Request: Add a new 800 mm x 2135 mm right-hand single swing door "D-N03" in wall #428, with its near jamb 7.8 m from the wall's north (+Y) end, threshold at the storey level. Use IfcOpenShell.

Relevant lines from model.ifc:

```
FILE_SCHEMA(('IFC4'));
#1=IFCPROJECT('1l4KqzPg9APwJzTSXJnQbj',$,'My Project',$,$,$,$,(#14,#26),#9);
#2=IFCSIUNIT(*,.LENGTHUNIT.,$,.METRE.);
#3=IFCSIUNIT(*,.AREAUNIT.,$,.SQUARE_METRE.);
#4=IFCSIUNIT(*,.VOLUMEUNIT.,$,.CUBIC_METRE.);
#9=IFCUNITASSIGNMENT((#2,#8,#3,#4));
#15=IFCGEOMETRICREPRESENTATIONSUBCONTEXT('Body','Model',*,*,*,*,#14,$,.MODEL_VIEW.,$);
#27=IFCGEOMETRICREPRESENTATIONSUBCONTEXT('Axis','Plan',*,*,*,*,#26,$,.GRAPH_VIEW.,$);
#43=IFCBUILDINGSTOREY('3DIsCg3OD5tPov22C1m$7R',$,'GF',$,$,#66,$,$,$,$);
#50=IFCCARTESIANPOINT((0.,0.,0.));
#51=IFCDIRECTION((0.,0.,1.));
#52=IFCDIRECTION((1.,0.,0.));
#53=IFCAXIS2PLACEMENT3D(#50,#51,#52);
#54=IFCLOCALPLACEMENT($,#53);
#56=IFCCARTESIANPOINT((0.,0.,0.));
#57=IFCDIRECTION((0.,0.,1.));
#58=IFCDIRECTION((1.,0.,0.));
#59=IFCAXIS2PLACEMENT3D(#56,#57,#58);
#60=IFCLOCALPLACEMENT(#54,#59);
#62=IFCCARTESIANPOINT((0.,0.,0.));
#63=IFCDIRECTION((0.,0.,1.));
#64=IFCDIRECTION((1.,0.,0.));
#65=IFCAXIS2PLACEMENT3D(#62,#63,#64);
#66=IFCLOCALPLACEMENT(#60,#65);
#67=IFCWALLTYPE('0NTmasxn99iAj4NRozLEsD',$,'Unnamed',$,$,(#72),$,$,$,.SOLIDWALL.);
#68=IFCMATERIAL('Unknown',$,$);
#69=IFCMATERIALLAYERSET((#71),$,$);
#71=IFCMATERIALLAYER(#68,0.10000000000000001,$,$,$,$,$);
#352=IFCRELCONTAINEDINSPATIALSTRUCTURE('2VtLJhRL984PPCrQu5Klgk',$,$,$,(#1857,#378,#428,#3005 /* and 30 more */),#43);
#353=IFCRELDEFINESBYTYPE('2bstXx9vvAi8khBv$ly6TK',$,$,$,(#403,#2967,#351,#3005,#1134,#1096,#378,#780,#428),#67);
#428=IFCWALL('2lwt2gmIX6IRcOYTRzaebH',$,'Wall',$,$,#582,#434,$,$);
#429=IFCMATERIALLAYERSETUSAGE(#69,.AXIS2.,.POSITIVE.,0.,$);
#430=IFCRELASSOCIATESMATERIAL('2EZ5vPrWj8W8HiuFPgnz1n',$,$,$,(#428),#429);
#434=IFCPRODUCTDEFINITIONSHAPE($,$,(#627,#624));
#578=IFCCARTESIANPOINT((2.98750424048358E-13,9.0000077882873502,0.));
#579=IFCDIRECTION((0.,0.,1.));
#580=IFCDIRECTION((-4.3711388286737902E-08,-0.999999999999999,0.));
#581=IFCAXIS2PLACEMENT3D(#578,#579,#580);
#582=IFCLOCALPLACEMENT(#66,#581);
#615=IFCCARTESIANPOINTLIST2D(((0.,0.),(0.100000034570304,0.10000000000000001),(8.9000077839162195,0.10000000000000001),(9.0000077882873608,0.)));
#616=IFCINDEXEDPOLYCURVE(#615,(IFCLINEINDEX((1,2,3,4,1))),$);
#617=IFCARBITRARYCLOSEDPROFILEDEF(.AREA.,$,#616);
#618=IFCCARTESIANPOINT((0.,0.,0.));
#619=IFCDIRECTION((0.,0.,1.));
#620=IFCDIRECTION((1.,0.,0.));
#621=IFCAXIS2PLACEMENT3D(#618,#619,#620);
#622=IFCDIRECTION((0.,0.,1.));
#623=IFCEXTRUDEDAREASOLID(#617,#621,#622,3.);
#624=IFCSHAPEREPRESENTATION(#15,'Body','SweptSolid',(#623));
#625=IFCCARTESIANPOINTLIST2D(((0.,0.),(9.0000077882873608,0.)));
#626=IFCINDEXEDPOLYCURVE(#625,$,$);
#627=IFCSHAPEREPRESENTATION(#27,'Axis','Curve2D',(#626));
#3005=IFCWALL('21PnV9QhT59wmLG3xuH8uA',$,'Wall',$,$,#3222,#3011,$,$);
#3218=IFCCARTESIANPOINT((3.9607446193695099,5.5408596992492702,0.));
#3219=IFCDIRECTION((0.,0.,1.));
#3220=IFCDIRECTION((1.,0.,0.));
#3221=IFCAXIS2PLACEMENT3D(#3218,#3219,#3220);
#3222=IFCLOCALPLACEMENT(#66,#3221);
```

```python
import numpy as np
import ifcopenshell
import ifcopenshell.api.feature
import ifcopenshell.api.geometry
import ifcopenshell.api.root
import ifcopenshell.api.spatial
import ifcopenshell.geom
import ifcopenshell.util.element
import ifcopenshell.util.placement
import ifcopenshell.util.representation
import ifcopenshell.util.shape
import ifcopenshell.util.unit

model = ifcopenshell.open("model.ifc")
unit_scale = ifcopenshell.util.unit.calculate_unit_scale(model)
settings = ifcopenshell.geom.settings()


def volume(element):
    """Net volume in cubic metres, openings subtracted."""
    shape = ifcopenshell.geom.create_shape(settings, element)
    return ifcopenshell.util.shape.get_volume(shape.geometry)


wall = model.by_id(428)
storey = ifcopenshell.util.element.get_container(wall, ifc_class="IfcBuildingStorey")
context = ifcopenshell.util.representation.get_context(model, "Model", "Body", "MODEL_VIEW")
before = volume(wall)

width, height, from_end, sill = 0.8, 2.135, 7.8, 0.0  # metres

# The wall runs along its own X axis, and the end named is its -X end.
wall_shape = ifcopenshell.geom.create_shape(settings, wall)
x, y, z = ifcopenshell.util.shape.get_vertices(wall_shape.geometry).T
start = x.min() + from_end
face, thickness = float(y.min()), float(y.max() - y.min())
wall_matrix = ifcopenshell.util.placement.get_local_placement(wall.ObjectPlacement)
level = ifcopenshell.util.placement.get_local_placement(storey.ObjectPlacement)[2, 3]


def in_wall(x, y):
    """Placement at x, y metres in the wall's axes, at sill height."""
    matrix = wall_matrix.copy()
    matrix[:, 3] = wall_matrix @ np.array([x / unit_scale, y / unit_scale, 0.0, 1.0])
    matrix[2, 3] = level + sill / unit_scale
    return matrix


# Opening: a box that overshoots both wall faces by 50 mm.
opening = ifcopenshell.api.root.create_entity(model, ifc_class="IfcOpeningElement", predefined_type="OPENING")
box = ifcopenshell.api.geometry.add_wall_representation(
    model, context=context, length=width, height=height, thickness=thickness + 0.1
)
ifcopenshell.api.geometry.assign_representation(model, product=opening, representation=box)
ifcopenshell.api.geometry.edit_object_placement(model, product=opening, matrix=in_wall(start, face - 0.05), is_si=False)
ifcopenshell.api.feature.add_feature(model, feature=opening, element=wall)

door = ifcopenshell.api.root.create_entity(model, ifc_class="IfcDoor", name="D-N03", predefined_type="DOOR")
door.OverallWidth, door.OverallHeight = width / unit_scale, height / unit_scale
door.OperationType = "SINGLE_SWING_RIGHT"
body = ifcopenshell.api.geometry.add_door_representation(
    model,
    context=context,
    overall_width=door.OverallWidth,
    overall_height=door.OverallHeight,
    operation_type="SINGLE_SWING_RIGHT",
    lining_properties={"LiningDepth": thickness / unit_scale, "ThresholdDepth": thickness / unit_scale},
)
ifcopenshell.api.geometry.assign_representation(model, product=door, representation=body)
ifcopenshell.api.spatial.assign_container(model, products=[door], relating_structure=storey)
ifcopenshell.api.feature.add_filling(model, opening=opening, element=door)

# The lining spans the wall, so the door starts at the wall face.
ifcopenshell.api.geometry.edit_object_placement(model, product=door, matrix=in_wall(start, face), is_si=False)

after = volume(wall)

print(f"wall volume {before:.3f} -> {after:.3f} m3")

model.write("model_rev.ifc")
```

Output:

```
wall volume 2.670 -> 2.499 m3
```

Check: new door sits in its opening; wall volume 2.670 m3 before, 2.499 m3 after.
